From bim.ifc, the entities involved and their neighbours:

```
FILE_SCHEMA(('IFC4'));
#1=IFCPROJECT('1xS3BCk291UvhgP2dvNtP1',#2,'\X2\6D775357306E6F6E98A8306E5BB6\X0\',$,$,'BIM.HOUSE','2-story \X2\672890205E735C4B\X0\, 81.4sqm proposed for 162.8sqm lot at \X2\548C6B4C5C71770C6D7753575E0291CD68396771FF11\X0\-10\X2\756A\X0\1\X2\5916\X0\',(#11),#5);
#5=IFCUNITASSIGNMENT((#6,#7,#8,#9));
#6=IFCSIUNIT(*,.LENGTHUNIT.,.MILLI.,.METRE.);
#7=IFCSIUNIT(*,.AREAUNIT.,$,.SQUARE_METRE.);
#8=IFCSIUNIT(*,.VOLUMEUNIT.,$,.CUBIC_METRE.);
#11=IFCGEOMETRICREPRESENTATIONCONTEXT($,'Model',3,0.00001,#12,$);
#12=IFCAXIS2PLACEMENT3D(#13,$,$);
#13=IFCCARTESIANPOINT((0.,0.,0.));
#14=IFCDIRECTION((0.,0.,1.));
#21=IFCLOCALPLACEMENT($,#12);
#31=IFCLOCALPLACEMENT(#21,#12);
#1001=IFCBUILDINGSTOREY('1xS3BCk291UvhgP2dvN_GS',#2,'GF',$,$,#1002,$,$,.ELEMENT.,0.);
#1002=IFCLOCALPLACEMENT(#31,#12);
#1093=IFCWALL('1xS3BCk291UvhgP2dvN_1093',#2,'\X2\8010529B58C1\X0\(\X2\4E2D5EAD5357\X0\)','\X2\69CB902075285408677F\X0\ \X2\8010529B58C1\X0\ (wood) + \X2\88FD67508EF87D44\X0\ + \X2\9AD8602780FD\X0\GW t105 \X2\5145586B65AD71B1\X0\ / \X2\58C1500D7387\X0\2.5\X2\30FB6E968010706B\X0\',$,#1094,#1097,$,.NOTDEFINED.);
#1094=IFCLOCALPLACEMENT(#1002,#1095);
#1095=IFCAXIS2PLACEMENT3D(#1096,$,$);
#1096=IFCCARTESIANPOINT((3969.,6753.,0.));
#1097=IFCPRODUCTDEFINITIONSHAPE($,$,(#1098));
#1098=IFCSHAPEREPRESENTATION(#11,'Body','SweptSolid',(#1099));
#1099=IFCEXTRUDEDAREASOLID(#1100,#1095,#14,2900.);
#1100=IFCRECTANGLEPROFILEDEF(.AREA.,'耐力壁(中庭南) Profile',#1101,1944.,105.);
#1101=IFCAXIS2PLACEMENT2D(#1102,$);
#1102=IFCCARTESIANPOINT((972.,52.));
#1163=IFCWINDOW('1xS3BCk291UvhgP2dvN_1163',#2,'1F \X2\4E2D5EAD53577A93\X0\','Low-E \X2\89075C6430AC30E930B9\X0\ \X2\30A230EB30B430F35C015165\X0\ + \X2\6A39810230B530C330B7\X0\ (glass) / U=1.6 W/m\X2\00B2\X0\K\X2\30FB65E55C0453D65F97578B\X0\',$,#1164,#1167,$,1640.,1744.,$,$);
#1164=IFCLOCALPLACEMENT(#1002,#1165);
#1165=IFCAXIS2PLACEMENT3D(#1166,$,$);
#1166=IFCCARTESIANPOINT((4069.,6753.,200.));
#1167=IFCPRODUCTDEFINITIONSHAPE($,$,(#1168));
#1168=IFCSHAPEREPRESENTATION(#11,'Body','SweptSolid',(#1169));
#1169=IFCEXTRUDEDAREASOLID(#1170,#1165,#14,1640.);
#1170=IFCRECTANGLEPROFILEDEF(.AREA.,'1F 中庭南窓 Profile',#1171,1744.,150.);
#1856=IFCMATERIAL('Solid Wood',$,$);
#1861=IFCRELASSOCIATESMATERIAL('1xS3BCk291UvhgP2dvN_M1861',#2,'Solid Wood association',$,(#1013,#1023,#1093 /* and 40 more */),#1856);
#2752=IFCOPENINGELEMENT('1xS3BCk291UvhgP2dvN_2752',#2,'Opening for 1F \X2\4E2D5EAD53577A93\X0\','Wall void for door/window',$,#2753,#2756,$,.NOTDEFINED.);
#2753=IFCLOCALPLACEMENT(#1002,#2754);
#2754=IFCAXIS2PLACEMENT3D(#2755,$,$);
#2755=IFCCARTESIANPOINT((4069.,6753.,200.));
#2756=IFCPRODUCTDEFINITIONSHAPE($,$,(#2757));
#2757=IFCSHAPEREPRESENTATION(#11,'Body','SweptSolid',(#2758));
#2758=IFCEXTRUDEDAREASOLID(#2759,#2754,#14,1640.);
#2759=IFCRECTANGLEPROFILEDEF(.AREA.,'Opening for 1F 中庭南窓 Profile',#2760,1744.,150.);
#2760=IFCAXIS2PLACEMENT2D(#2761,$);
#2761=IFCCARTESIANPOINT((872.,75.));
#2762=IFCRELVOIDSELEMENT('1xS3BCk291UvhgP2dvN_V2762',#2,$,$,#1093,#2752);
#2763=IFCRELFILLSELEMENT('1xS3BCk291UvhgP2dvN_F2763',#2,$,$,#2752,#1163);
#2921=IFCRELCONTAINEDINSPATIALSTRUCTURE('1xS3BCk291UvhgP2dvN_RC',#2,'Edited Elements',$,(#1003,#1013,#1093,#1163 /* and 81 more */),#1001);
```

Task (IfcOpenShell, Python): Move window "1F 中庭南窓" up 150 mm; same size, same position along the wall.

```python
import numpy as np
import ifcopenshell
import ifcopenshell.api.geometry
import ifcopenshell.util.placement
import ifcopenshell.util.unit

model = ifcopenshell.open("bim.ifc")
unit_scale = ifcopenshell.util.unit.calculate_unit_scale(model)

window = model.by_id(1163)
opening = window.FillsVoids[0].RelatingOpeningElement
dz = 0.15 / unit_scale

shift = np.array([0.0, 0.0, dz])
# The window is not placed relative to its opening, so move both.
for product in (opening, window):
    matrix = ifcopenshell.util.placement.get_local_placement(product.ObjectPlacement)
    matrix[:3, 3] += shift
    ifcopenshell.api.geometry.edit_object_placement(model, product=product, matrix=matrix, is_si=False)

print(f"moved by {dz * unit_scale:+.3f} m")

model.write("bim_rev.ifc")
```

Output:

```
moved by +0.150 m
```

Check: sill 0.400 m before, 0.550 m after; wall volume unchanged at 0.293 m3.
